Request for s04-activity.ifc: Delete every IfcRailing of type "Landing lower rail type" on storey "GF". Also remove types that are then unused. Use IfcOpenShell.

First a look at what the model holds.

```python
import ifcopenshell
import ifcopenshell.util.element

model = ifcopenshell.open("s04-activity.ifc")
print(model.schema)
storey = next(s for s in model.by_type("IfcBuildingStorey") if s.Name == "GF")
railings = [e for e in ifcopenshell.util.element.get_decomposition(storey) if e.is_a("IfcRailing")]
seen = {}
for e in railings:
    element_type = ifcopenshell.util.element.get_type(e)
    name = element_type.Name if element_type not in (None, e) else None
    seen[name] = seen.get(name, 0) + 1
for name, count in sorted(seen.items(), key=str):
    print(count, "x", name)
```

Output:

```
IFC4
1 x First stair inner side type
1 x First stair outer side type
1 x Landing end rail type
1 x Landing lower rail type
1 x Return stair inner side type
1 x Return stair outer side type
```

```python
import ifcopenshell
import ifcopenshell.api.root
import ifcopenshell.util.element

model = ifcopenshell.open("s04-activity.ifc")

storey = next(s for s in model.by_type("IfcBuildingStorey") if s.Name == "GF")
railings = [e for e in ifcopenshell.util.element.get_decomposition(storey) if e.is_a("IfcRailing")]
targets = [e for e in railings if (t := ifcopenshell.util.element.get_type(e)) not in (None, e) and t.Name == "Landing lower rail type"]
types = {ifcopenshell.util.element.get_type(e) for e in targets} - {None, *targets}

for e in targets:
    ifcopenshell.api.root.remove_product(model, product=e)
print(len(targets), "removed")

unused = [t for t in types if not ifcopenshell.util.element.get_types(t)]
for t in unused:
    ifcopenshell.api.root.remove_product(model, product=t)
print(len(unused), "unused types removed")

model.write("s04-activity_updated.ifc")
```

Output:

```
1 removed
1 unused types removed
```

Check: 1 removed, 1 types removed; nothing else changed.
